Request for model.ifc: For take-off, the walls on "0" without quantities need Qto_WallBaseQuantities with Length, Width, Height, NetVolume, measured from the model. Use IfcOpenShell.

First a look at what the model holds.

```python
import ifcopenshell
import ifcopenshell.util.element
import ifcopenshell.util.unit

model = ifcopenshell.open("model.ifc")
print(model.schema)
for unit_type in ("LENGTHUNIT", "AREAUNIT", "VOLUMEUNIT"):
    print(unit_type, ifcopenshell.util.unit.calculate_unit_scale(model, unit_type))
storey = next(s for s in model.by_type("IfcBuildingStorey") if s.Name == "0")
walls = [e for e in ifcopenshell.util.element.get_decomposition(storey) if e.is_a("IfcWall")]
for e in sorted(walls, key=lambda e: e.id()):
    print(e.id(), e.is_a(), e.Name, list(ifcopenshell.util.element.get_psets(e, qtos_only=True)), sep=" | ")
```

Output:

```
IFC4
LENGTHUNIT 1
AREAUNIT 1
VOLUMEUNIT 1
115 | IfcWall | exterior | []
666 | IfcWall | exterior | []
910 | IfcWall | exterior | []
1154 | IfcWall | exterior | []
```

```python
import ifcopenshell
import ifcopenshell.api.pset
import ifcopenshell.geom
import ifcopenshell.util.element
import ifcopenshell.util.shape
import ifcopenshell.util.unit

model = ifcopenshell.open("model.ifc")
unit_scale = ifcopenshell.util.unit.calculate_unit_scale(model)
volume_scale = ifcopenshell.util.unit.calculate_unit_scale(model, "VOLUMEUNIT")
settings = ifcopenshell.geom.settings()

storey = next(s for s in model.by_type("IfcBuildingStorey") if s.Name == "0")
walls = [e for e in ifcopenshell.util.element.get_decomposition(storey) if e.is_a("IfcWall")]

for e in sorted(walls, key=lambda e: e.id()):
    if ifcopenshell.util.element.get_psets(e, qtos_only=True, should_inherit=False):
        continue
    # Geometry comes back in metres, in the element's own axes.
    shape = ifcopenshell.geom.create_shape(settings, e)
    values = {
        "Length": ifcopenshell.util.shape.get_x(shape.geometry) / unit_scale,
        "Width": ifcopenshell.util.shape.get_y(shape.geometry) / unit_scale,
        "Height": ifcopenshell.util.shape.get_z(shape.geometry) / unit_scale,
        "NetVolume": ifcopenshell.util.shape.get_volume(shape.geometry) / volume_scale,
    }
    qto = ifcopenshell.api.pset.add_qto(model, product=e, name="Qto_WallBaseQuantities")
    ifcopenshell.api.pset.edit_qto(model, qto=qto, properties=values)
    print(e.id(), {k: round(v, 3) for k, v in values.items()})

model.write("model_rev.ifc")
```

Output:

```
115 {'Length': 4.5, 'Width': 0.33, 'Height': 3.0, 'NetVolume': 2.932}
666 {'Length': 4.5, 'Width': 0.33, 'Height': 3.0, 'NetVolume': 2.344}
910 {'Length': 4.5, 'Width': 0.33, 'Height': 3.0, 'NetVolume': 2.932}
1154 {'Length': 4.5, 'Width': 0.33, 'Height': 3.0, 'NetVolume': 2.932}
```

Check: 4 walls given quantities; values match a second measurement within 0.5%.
